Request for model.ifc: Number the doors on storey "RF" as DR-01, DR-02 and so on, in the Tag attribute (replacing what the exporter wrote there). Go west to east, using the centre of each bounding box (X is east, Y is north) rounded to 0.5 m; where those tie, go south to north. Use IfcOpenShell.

First a look at what the model holds.

```python
import ifcopenshell
import ifcopenshell.util.element
import ifcopenshell.util.placement

model = ifcopenshell.open("model.ifc")
print(model.schema)
storey = next(s for s in model.by_type("IfcBuildingStorey") if s.Name == "RF")
doors = [e for e in ifcopenshell.util.element.get_decomposition(storey) if e.is_a("IfcDoor")]
for e in sorted(doors, key=lambda e: e.id()):
    origin = ifcopenshell.util.placement.get_local_placement(e.ObjectPlacement)[:3, 3]
    print(e.id(), e.Tag, e.Name, origin.round(2) + 0.0, sep=" | ")
```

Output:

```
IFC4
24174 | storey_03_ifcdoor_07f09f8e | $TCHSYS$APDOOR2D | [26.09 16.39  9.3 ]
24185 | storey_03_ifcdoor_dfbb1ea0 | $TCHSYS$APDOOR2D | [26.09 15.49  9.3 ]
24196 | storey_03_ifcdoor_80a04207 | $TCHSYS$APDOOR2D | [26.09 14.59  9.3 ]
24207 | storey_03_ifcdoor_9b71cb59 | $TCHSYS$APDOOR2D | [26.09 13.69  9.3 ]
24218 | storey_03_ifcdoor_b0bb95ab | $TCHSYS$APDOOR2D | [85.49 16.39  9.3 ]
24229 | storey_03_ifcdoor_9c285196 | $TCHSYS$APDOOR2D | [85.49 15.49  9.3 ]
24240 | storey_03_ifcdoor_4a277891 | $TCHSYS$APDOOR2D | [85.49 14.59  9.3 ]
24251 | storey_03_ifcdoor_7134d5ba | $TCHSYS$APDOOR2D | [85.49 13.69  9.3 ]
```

```python
import ifcopenshell
import ifcopenshell.geom
import ifcopenshell.util.element
import ifcopenshell.util.shape

model = ifcopenshell.open("model.ifc")
settings = ifcopenshell.geom.settings()
settings.set("use-world-coords", True)


def centre(element):
    shape = ifcopenshell.geom.create_shape(settings, element)
    return ifcopenshell.util.shape.get_bbox_centroid(shape.geometry)


storey = next(s for s in model.by_type("IfcBuildingStorey") if s.Name == "RF")
doors = [e for e in ifcopenshell.util.element.get_decomposition(storey) if e.is_a("IfcDoor")]

# Insertion points can sit at a corner or the storey origin, so sort by the geometry (in metres).
centres = {e: centre(e) for e in doors}
doors.sort(key=lambda e: (round(centres[e][0] / 0.5), centres[e][1]))

for i, e in enumerate(doors, start=1):
    number = f"DR-{i:02d}"
    e.Tag = number
    print(e.id(), number)

model.write("model-out.ifc")
```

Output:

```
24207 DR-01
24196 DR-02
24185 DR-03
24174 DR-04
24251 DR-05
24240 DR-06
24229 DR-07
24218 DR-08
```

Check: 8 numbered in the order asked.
